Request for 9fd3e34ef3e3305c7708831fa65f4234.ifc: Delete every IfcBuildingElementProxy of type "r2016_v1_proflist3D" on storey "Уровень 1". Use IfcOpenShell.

First a look at what the model holds.

```python
import ifcopenshell
import ifcopenshell.util.element

model = ifcopenshell.open("9fd3e34ef3e3305c7708831fa65f4234.ifc")
print(model.schema)
storey = next(s for s in model.by_type("IfcBuildingStorey") if s.Name == "Уровень 1")
proxies = [e for e in ifcopenshell.util.element.get_decomposition(storey) if e.is_a("IfcBuildingElementProxy")]
seen = {}
for e in proxies:
    element_type = ifcopenshell.util.element.get_type(e)
    name = element_type.Name if element_type not in (None, e) else None
    seen[name] = seen.get(name, 0) + 1
for name, count in sorted(seen.items(), key=str):
    print(count, "x", name)
```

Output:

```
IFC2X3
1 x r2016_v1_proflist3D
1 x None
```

```python
import ifcopenshell
import ifcopenshell.api.root
import ifcopenshell.util.element

model = ifcopenshell.open("9fd3e34ef3e3305c7708831fa65f4234.ifc")

storey = next(s for s in model.by_type("IfcBuildingStorey") if s.Name == "Уровень 1")
proxies = [e for e in ifcopenshell.util.element.get_decomposition(storey) if e.is_a("IfcBuildingElementProxy")]
targets = [e for e in proxies if (t := ifcopenshell.util.element.get_type(e)) not in (None, e) and t.Name == "r2016_v1_proflist3D"]

for e in targets:
    ifcopenshell.api.root.remove_product(model, product=e)
print(len(targets), "removed")

model.write("9fd3e34ef3e3305c7708831fa65f4234_v2.ifc")
```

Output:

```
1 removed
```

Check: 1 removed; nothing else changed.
